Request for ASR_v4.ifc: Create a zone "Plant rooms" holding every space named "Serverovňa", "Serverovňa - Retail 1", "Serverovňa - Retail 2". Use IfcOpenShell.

First a look at what the model holds.

```python
import ifcopenshell

model = ifcopenshell.open("ASR_v4.ifc")
print(model.schema)
seen = {}
for space in model.by_type("IfcSpace"):
    seen[space.LongName] = seen.get(space.LongName, 0) + 1
for name, count in sorted(seen.items(), key=str):
    print(count, "x", name)
print("zones:", [z.Name for z in model.by_type("IfcZone")][:20])
```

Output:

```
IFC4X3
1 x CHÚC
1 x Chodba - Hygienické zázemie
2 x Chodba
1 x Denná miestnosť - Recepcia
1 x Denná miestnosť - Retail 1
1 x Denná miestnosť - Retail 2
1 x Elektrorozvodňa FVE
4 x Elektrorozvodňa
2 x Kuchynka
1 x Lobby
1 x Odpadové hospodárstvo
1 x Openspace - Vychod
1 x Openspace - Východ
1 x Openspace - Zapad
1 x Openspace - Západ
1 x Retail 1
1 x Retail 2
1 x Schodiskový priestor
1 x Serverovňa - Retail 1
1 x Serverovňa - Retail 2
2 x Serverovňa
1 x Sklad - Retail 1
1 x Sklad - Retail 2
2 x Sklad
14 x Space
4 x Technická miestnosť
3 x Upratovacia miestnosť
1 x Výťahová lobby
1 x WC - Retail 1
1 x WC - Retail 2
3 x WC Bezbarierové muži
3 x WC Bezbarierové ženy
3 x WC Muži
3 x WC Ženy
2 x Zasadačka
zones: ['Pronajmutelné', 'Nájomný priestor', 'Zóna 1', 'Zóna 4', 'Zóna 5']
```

```python
import ifcopenshell
import ifcopenshell.api.group
import ifcopenshell.api.root

model = ifcopenshell.open("ASR_v4.ifc")

names = {"Serverovňa", "Serverovňa - Retail 1", "Serverovňa - Retail 2"}
spaces = [s for s in model.by_type("IfcSpace") if s.LongName in names]

zone = ifcopenshell.api.root.create_entity(model, ifc_class="IfcZone", name="Plant rooms")
ifcopenshell.api.group.assign_group(model, products=spaces, group=zone)
print(len(spaces), "spaces in", zone.Name)

model.write("ASR_v4_v2.ifc")
```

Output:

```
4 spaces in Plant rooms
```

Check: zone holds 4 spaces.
